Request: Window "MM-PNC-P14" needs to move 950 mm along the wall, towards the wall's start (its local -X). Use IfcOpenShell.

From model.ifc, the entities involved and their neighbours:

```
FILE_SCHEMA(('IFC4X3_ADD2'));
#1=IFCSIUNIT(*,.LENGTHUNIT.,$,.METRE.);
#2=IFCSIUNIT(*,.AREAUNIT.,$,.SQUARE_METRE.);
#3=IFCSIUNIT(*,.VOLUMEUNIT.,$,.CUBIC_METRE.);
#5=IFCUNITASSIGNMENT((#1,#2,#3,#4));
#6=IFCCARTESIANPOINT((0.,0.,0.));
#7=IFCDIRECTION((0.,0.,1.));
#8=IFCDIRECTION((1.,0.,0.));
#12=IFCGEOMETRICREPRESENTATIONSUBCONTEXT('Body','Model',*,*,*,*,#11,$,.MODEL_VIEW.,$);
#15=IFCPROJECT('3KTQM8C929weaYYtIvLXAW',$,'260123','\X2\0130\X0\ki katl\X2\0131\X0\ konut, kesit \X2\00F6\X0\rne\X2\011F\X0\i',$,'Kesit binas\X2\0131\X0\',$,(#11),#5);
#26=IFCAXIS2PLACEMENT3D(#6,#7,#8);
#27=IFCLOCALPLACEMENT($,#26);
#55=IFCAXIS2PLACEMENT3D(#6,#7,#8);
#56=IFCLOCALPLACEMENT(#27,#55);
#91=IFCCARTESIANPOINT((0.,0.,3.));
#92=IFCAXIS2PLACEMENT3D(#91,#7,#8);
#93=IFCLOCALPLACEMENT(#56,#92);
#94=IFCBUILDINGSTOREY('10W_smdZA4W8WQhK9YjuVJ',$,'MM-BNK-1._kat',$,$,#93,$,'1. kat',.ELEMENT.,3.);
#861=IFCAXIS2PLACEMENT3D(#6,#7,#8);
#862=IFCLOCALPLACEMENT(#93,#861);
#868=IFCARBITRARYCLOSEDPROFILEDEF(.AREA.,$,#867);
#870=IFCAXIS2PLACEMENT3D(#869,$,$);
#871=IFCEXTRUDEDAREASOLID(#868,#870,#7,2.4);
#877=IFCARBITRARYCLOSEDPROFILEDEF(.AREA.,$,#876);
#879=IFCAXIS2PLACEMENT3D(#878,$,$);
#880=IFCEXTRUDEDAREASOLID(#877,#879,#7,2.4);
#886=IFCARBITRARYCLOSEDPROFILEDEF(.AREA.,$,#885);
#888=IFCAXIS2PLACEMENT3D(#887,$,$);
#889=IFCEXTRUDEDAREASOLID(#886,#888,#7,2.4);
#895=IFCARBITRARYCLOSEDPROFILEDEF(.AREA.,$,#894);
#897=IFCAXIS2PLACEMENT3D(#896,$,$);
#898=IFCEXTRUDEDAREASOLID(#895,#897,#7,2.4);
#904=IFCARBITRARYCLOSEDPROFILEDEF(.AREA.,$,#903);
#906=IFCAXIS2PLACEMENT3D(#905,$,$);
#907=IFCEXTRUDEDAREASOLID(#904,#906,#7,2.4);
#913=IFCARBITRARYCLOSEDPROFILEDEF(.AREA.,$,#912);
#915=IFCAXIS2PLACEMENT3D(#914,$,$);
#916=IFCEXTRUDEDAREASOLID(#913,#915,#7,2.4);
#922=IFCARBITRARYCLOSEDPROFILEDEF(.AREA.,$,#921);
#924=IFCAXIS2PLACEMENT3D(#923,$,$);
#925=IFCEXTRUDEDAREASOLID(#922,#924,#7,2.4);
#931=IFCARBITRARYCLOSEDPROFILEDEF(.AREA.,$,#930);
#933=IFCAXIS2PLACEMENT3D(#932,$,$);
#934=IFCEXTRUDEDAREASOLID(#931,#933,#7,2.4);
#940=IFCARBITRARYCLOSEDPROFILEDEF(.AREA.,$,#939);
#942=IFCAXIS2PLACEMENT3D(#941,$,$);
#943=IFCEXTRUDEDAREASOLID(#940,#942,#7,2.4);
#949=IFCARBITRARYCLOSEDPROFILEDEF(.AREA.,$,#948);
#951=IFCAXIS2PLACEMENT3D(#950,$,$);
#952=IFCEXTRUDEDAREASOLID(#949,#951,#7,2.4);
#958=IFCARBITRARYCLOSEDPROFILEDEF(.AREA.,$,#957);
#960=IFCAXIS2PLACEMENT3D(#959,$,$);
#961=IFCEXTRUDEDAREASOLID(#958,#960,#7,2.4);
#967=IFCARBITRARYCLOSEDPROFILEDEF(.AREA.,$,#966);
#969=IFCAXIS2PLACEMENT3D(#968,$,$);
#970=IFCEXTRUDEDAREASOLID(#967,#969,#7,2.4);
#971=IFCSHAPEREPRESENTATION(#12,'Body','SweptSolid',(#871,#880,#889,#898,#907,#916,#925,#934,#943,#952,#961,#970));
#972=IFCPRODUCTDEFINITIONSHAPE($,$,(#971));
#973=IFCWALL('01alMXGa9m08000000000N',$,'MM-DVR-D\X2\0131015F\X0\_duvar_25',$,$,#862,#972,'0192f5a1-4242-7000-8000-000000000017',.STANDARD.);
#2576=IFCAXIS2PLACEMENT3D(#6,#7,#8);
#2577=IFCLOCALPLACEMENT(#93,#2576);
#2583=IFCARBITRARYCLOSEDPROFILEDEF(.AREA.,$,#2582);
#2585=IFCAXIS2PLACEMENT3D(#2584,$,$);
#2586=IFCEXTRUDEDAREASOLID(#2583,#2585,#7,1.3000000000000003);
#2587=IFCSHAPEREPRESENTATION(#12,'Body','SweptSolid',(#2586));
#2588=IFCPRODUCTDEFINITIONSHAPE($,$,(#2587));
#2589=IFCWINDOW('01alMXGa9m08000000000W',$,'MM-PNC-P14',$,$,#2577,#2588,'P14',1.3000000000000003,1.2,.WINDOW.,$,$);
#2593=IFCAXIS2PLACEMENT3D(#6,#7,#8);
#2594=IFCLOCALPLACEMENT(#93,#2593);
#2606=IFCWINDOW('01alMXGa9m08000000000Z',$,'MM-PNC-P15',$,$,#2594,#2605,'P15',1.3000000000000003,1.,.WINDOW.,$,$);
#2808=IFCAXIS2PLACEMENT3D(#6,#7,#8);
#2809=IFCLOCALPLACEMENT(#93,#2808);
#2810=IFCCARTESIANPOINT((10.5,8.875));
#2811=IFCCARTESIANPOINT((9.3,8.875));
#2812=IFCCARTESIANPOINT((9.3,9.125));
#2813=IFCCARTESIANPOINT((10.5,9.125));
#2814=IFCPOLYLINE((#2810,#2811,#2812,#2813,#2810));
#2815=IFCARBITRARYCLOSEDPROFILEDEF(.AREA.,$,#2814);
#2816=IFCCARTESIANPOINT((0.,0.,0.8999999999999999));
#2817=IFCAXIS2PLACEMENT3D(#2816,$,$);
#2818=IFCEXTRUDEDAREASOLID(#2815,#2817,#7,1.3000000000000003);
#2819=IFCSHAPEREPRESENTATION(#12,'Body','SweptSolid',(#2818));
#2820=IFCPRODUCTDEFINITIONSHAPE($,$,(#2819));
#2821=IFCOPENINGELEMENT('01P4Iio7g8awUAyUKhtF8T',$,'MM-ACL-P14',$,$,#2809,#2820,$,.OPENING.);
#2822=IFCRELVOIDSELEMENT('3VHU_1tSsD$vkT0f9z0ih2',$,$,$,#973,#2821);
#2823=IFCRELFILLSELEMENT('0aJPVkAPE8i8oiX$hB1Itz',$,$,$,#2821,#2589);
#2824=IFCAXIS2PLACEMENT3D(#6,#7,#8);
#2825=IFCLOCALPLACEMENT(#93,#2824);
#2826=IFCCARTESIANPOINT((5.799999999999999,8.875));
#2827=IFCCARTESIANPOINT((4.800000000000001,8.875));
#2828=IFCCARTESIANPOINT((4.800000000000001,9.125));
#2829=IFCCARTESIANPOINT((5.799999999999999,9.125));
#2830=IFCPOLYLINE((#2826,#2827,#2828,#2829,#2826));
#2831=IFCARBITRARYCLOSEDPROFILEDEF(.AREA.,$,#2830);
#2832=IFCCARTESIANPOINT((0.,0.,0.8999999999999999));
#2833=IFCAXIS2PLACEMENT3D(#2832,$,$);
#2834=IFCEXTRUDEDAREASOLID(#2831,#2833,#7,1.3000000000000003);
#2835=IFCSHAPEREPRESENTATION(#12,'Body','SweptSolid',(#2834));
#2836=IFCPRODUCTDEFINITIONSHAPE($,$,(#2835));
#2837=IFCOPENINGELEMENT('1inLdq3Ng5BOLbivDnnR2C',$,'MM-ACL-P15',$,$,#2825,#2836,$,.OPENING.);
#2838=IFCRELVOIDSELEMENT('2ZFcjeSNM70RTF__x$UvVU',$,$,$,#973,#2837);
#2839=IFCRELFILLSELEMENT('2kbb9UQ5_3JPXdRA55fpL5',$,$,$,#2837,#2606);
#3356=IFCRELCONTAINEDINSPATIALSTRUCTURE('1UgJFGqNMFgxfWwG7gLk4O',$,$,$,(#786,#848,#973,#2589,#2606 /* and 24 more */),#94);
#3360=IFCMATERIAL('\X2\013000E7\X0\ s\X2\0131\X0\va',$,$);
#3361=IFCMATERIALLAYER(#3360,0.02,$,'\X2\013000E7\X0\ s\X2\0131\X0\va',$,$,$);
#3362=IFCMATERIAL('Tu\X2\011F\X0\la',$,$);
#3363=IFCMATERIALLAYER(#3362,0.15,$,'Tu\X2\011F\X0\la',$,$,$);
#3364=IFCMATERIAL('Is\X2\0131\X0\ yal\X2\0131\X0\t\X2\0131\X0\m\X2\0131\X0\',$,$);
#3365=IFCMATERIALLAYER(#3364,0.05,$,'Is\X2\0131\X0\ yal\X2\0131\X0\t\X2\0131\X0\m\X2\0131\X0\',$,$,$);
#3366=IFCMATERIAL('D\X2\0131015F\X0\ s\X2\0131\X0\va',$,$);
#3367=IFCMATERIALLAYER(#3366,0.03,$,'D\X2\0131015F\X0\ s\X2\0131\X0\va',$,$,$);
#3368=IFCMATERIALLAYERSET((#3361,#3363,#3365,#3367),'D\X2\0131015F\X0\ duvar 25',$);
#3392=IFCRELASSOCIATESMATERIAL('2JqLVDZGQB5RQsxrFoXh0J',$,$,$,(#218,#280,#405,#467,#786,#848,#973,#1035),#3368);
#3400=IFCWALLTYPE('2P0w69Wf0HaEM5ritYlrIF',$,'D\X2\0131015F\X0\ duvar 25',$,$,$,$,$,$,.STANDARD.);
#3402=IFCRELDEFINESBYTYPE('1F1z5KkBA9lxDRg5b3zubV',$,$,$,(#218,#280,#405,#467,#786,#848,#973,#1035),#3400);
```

```python
import ifcopenshell
import ifcopenshell.api.geometry
import ifcopenshell.util.placement

model = ifcopenshell.open("model.ifc")

window = model.by_guid("01alMXGa9m08000000000W")
opening = window.FillsVoids[0].RelatingOpeningElement
wall = opening.VoidsElements[0].RelatingBuildingElement

wall_matrix = ifcopenshell.util.placement.get_local_placement(wall.ObjectPlacement)
shift = wall_matrix[:3, 0] * -0.95
before = ifcopenshell.util.placement.get_local_placement(window.ObjectPlacement)[:3, 3].copy()

# The window is not placed relative to its opening, so move both.
for product in (opening, window):
    matrix = ifcopenshell.util.placement.get_local_placement(product.ObjectPlacement)
    matrix[:3, 3] += shift
    ifcopenshell.api.geometry.edit_object_placement(model, product=product, matrix=matrix, is_si=False)

after = ifcopenshell.util.placement.get_local_placement(window.ObjectPlacement)[:3, 3]
print("window moved by", (after - before).round(3) + 0.0)

model.write("model-out.ifc")
```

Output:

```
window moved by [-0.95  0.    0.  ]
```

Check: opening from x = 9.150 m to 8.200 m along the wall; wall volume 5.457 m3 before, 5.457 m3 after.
